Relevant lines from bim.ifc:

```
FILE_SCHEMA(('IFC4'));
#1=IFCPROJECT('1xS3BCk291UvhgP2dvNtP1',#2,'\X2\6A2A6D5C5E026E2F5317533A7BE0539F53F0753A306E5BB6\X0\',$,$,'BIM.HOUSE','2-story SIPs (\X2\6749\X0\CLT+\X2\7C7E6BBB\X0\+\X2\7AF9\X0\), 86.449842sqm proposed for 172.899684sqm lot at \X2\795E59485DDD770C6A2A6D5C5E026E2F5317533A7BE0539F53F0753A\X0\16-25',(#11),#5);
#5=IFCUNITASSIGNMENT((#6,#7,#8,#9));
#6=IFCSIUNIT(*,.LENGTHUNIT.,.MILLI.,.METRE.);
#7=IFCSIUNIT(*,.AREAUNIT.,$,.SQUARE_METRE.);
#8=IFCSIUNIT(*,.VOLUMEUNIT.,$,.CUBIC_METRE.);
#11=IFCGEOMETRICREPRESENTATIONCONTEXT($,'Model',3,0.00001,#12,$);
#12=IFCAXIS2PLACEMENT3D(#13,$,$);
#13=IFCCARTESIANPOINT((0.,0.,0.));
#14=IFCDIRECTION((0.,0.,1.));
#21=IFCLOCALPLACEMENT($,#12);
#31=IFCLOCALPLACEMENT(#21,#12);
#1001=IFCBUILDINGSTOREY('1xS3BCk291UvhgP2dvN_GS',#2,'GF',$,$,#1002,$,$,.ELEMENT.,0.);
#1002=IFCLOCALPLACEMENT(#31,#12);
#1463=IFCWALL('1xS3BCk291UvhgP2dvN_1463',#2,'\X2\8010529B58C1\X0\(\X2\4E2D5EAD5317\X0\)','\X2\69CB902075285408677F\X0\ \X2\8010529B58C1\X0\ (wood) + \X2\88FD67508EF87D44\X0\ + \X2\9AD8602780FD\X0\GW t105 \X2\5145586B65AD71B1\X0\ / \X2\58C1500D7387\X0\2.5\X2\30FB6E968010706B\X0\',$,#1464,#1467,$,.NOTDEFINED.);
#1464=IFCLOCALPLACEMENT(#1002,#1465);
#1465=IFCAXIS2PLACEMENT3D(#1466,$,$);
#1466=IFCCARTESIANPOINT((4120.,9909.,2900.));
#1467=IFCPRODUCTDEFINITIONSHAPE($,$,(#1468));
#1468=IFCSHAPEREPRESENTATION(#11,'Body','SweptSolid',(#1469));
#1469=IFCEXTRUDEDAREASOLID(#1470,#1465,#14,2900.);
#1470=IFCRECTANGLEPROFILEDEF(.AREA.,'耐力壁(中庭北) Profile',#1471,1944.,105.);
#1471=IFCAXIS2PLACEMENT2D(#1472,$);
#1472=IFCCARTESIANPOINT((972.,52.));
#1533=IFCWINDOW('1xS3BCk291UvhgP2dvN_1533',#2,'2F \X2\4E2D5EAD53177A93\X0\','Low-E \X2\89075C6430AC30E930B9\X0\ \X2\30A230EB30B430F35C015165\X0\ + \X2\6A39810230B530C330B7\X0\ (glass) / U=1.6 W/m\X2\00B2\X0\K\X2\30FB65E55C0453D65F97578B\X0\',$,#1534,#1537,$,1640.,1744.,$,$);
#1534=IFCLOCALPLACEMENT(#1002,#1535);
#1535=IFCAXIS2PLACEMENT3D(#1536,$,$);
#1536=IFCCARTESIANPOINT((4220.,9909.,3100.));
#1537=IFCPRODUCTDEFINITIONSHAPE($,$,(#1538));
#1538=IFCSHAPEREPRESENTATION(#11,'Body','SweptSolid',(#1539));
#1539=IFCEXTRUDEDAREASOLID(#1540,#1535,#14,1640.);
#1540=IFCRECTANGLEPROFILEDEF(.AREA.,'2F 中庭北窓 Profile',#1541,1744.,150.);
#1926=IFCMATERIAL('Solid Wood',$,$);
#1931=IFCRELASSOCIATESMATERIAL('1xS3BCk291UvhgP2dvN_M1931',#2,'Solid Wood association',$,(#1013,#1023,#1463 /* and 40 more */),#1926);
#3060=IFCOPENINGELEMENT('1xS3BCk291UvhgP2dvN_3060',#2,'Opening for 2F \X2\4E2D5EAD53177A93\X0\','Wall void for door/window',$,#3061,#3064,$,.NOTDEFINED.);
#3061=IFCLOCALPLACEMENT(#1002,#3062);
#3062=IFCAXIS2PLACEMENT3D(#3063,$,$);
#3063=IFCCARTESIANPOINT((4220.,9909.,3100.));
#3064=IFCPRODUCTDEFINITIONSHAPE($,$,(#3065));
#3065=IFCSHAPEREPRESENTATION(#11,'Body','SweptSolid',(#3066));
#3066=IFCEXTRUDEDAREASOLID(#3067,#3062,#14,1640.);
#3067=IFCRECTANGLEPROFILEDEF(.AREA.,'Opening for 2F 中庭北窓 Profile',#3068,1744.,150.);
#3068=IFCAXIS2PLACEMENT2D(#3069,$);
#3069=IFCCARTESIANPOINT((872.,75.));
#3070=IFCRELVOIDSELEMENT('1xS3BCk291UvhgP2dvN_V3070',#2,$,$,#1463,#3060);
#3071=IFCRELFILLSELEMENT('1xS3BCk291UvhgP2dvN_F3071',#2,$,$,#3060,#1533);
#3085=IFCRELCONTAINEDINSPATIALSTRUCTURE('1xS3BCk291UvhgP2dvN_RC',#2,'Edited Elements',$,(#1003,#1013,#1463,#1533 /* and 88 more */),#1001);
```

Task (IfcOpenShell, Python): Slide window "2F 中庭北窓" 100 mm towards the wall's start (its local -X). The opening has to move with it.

```python
import ifcopenshell
import ifcopenshell.api.geometry
import ifcopenshell.util.placement
import ifcopenshell.util.unit

model = ifcopenshell.open("bim.ifc")
unit_scale = ifcopenshell.util.unit.calculate_unit_scale(model)

window = model.by_guid("1xS3BCk291UvhgP2dvN_1533")
opening = window.FillsVoids[0].RelatingOpeningElement
wall = opening.VoidsElements[0].RelatingBuildingElement

wall_matrix = ifcopenshell.util.placement.get_local_placement(wall.ObjectPlacement)
shift = wall_matrix[:3, 0] * -0.1 / unit_scale
before = ifcopenshell.util.placement.get_local_placement(window.ObjectPlacement)[:3, 3].copy()

# The window is not placed relative to its opening, so move both.
for product in (opening, window):
    matrix = ifcopenshell.util.placement.get_local_placement(product.ObjectPlacement)
    matrix[:3, 3] += shift
    ifcopenshell.api.geometry.edit_object_placement(model, product=product, matrix=matrix, is_si=False)

after = ifcopenshell.util.placement.get_local_placement(window.ObjectPlacement)[:3, 3]
print("window moved by", (after - before).round(3) + 0.0)

model.write("bim-out.ifc")
```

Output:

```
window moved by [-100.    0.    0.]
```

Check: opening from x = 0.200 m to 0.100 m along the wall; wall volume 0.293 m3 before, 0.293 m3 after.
